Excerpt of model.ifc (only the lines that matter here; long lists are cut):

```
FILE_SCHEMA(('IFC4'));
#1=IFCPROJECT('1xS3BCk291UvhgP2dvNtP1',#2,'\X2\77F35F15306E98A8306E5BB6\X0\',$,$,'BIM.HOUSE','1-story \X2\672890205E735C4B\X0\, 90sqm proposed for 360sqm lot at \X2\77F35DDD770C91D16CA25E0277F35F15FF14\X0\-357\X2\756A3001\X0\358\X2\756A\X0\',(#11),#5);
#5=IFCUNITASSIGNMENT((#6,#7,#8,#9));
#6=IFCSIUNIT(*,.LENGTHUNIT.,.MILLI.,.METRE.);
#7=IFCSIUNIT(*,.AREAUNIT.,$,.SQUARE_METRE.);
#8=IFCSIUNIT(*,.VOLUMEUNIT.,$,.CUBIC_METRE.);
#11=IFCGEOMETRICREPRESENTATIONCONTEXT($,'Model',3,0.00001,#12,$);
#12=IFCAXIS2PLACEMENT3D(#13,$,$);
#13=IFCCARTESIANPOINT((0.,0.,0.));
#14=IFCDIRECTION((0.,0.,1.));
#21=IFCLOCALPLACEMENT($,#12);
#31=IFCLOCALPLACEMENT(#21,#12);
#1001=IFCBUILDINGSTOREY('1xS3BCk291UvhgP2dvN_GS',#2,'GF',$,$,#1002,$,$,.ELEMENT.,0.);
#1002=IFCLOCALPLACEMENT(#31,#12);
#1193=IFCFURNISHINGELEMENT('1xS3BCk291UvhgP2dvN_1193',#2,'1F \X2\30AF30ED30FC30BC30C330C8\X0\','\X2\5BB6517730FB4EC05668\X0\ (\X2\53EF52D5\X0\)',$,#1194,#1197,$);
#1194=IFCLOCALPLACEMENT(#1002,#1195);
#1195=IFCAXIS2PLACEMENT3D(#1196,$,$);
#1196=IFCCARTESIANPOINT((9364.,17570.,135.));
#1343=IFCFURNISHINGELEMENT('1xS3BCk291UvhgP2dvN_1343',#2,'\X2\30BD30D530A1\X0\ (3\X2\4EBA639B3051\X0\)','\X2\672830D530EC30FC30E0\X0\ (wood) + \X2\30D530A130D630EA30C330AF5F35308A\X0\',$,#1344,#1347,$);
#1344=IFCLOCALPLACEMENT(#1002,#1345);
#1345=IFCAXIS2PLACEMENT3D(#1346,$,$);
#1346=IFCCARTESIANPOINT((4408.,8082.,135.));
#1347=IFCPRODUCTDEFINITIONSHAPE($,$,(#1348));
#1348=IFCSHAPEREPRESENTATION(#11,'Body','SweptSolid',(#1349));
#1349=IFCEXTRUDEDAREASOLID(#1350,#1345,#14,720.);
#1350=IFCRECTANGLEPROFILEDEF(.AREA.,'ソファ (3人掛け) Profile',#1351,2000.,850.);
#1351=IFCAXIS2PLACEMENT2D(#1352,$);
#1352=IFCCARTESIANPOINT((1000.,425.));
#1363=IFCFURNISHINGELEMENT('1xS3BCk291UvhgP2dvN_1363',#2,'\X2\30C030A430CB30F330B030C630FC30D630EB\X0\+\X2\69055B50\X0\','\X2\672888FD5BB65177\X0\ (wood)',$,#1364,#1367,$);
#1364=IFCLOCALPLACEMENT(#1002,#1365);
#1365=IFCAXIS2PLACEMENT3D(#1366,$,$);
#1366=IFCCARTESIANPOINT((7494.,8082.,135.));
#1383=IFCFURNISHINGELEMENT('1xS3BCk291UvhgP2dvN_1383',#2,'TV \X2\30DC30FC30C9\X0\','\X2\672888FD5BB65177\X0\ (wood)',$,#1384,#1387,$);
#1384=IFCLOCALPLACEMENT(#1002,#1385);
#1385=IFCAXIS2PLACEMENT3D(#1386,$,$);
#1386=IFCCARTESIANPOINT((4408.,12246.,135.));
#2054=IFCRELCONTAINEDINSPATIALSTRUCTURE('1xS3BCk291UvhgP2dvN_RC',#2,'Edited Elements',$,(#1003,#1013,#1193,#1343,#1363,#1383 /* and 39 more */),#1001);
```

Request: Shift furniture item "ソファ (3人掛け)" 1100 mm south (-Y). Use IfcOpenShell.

```python
import ifcopenshell
import ifcopenshell.api.geometry
import ifcopenshell.util.placement
import ifcopenshell.util.unit

model = ifcopenshell.open("model.ifc")
unit_scale = ifcopenshell.util.unit.calculate_unit_scale(model)

item = model.by_guid("1xS3BCk291UvhgP2dvN_1343")
matrix = ifcopenshell.util.placement.get_local_placement(item.ObjectPlacement)
matrix[1, 3] -= 1.1 / unit_scale
ifcopenshell.api.geometry.edit_object_placement(model, product=item, matrix=matrix, is_si=False)

print(ifcopenshell.util.placement.get_local_placement(item.ObjectPlacement).round(3) + 0.0)

model.write("model_rev.ifc")
```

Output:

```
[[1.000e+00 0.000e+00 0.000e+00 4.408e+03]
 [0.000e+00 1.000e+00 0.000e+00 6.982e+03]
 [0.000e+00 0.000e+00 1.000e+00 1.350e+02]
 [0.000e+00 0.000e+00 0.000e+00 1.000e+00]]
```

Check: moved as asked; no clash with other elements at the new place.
